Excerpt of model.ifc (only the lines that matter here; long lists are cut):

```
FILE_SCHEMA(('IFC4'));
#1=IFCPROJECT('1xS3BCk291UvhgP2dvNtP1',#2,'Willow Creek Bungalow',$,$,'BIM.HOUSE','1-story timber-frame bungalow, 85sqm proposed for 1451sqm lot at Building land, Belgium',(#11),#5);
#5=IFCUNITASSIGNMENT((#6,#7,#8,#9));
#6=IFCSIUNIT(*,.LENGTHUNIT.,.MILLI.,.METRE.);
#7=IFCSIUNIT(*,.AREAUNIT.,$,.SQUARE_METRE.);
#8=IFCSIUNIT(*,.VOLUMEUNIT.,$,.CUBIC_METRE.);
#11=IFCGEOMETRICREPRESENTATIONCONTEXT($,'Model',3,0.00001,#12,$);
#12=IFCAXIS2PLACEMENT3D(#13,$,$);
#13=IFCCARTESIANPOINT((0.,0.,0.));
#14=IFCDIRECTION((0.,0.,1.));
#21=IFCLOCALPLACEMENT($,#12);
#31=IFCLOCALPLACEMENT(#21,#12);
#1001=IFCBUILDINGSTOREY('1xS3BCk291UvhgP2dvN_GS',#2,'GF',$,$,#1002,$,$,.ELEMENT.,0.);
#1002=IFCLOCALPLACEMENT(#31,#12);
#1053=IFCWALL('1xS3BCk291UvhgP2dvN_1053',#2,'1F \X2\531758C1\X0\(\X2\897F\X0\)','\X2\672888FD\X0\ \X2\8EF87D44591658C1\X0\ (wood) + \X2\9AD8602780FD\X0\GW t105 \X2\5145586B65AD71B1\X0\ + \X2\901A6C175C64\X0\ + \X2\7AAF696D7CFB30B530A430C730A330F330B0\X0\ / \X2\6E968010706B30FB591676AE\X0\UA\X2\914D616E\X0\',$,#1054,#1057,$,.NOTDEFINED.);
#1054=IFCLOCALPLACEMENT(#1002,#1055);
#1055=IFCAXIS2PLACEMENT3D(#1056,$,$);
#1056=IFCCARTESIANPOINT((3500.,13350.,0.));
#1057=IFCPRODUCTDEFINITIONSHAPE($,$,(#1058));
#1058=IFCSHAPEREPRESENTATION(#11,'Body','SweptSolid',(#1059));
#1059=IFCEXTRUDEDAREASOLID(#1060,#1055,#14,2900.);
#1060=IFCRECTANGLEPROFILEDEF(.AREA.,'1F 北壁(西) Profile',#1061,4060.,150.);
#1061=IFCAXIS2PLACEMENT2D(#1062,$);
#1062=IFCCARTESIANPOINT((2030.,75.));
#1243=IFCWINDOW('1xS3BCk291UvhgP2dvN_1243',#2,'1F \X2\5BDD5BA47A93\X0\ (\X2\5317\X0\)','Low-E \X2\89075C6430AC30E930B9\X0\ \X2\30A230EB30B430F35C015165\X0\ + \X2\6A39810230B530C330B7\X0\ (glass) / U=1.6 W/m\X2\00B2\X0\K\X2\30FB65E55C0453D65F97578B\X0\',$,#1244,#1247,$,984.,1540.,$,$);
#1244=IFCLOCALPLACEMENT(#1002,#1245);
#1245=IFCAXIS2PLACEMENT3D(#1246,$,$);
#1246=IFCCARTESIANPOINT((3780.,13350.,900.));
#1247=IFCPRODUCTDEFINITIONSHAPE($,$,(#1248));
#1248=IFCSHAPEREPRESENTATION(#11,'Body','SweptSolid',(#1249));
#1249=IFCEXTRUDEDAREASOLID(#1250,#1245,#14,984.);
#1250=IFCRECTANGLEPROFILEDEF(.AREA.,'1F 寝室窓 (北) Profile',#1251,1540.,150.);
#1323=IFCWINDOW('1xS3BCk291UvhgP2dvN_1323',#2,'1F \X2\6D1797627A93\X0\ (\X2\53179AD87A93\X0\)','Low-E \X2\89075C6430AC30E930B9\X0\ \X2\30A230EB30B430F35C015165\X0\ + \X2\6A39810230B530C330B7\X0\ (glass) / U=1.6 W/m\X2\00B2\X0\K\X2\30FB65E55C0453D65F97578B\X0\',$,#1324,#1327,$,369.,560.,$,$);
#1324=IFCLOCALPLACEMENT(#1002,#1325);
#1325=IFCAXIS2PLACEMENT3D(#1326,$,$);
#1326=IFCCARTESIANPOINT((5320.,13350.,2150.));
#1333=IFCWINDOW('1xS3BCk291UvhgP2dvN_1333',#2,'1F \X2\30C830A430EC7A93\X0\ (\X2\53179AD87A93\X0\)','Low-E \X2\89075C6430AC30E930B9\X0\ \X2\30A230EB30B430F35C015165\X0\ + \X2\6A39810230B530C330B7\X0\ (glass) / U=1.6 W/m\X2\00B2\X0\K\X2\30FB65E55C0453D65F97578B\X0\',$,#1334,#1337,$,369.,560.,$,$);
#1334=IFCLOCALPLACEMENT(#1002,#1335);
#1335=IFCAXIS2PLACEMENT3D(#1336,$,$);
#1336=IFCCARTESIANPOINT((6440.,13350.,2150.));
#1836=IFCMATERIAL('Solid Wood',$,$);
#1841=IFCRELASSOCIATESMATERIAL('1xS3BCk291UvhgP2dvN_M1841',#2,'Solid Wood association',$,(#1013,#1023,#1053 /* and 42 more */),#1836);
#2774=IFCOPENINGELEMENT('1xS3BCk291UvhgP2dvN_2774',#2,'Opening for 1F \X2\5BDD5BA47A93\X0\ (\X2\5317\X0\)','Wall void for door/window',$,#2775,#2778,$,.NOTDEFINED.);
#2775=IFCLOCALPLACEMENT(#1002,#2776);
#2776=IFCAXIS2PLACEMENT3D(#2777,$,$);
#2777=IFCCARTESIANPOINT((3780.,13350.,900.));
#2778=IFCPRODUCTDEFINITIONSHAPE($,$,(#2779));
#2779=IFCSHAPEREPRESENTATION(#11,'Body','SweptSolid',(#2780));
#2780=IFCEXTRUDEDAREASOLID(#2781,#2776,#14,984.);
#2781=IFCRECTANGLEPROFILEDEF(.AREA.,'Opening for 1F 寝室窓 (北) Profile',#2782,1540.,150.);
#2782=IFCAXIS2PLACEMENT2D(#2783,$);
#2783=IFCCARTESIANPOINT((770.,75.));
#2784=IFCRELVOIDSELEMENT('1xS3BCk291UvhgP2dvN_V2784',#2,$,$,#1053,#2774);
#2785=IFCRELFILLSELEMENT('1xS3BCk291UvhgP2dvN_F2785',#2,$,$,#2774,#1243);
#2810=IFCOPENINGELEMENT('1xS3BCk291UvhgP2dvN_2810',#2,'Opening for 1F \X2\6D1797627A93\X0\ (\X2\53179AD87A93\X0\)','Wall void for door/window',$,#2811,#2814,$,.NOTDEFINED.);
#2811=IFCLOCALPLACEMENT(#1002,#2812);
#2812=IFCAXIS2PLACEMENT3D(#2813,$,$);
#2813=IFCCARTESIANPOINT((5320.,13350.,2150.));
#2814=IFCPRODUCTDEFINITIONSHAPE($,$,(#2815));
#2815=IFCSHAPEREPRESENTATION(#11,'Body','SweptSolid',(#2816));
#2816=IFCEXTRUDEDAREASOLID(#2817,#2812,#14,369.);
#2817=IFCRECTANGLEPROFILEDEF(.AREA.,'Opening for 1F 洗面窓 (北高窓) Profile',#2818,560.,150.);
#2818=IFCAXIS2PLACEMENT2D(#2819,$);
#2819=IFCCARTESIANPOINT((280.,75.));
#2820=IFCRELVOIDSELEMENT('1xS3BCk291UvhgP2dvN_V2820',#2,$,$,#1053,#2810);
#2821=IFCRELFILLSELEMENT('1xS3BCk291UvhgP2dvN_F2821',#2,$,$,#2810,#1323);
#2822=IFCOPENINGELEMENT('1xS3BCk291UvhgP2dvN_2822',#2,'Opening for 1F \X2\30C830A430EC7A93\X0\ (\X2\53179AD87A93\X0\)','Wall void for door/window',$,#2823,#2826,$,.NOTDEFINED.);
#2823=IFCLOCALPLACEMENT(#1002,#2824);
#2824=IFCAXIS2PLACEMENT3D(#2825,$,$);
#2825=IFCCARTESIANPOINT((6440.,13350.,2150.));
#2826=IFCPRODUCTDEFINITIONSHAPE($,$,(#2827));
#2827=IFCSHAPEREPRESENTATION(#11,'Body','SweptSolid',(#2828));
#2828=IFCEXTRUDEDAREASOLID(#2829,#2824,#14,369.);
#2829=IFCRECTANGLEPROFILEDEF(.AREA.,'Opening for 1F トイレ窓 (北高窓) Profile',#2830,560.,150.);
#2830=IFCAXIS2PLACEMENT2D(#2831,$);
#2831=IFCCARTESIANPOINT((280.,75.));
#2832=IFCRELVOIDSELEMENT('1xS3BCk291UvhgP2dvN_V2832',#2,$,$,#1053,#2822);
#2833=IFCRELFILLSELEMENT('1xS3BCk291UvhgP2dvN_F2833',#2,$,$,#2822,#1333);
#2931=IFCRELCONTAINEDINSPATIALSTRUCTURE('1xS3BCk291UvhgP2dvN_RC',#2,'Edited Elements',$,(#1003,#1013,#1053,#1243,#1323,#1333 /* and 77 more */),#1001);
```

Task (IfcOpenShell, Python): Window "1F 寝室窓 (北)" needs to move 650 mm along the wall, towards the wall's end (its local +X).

```python
import ifcopenshell
import ifcopenshell.api.geometry
import ifcopenshell.util.placement
import ifcopenshell.util.unit

model = ifcopenshell.open("model.ifc")
unit_scale = ifcopenshell.util.unit.calculate_unit_scale(model)

window = model.by_guid("1xS3BCk291UvhgP2dvN_1243")
opening = window.FillsVoids[0].RelatingOpeningElement
wall = opening.VoidsElements[0].RelatingBuildingElement

wall_matrix = ifcopenshell.util.placement.get_local_placement(wall.ObjectPlacement)
shift = wall_matrix[:3, 0] * 0.65 / unit_scale
before = ifcopenshell.util.placement.get_local_placement(window.ObjectPlacement)[:3, 3].copy()

# The window is not placed relative to its opening, so move both.
for product in (opening, window):
    matrix = ifcopenshell.util.placement.get_local_placement(product.ObjectPlacement)
    matrix[:3, 3] += shift
    ifcopenshell.api.geometry.edit_object_placement(model, product=product, matrix=matrix, is_si=False)

after = ifcopenshell.util.placement.get_local_placement(window.ObjectPlacement)[:3, 3]
print("window moved by", (after - before).round(3) + 0.0)

model.write("model_updated.ifc")
```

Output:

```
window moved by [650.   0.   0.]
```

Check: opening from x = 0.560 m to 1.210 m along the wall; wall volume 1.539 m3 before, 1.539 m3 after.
